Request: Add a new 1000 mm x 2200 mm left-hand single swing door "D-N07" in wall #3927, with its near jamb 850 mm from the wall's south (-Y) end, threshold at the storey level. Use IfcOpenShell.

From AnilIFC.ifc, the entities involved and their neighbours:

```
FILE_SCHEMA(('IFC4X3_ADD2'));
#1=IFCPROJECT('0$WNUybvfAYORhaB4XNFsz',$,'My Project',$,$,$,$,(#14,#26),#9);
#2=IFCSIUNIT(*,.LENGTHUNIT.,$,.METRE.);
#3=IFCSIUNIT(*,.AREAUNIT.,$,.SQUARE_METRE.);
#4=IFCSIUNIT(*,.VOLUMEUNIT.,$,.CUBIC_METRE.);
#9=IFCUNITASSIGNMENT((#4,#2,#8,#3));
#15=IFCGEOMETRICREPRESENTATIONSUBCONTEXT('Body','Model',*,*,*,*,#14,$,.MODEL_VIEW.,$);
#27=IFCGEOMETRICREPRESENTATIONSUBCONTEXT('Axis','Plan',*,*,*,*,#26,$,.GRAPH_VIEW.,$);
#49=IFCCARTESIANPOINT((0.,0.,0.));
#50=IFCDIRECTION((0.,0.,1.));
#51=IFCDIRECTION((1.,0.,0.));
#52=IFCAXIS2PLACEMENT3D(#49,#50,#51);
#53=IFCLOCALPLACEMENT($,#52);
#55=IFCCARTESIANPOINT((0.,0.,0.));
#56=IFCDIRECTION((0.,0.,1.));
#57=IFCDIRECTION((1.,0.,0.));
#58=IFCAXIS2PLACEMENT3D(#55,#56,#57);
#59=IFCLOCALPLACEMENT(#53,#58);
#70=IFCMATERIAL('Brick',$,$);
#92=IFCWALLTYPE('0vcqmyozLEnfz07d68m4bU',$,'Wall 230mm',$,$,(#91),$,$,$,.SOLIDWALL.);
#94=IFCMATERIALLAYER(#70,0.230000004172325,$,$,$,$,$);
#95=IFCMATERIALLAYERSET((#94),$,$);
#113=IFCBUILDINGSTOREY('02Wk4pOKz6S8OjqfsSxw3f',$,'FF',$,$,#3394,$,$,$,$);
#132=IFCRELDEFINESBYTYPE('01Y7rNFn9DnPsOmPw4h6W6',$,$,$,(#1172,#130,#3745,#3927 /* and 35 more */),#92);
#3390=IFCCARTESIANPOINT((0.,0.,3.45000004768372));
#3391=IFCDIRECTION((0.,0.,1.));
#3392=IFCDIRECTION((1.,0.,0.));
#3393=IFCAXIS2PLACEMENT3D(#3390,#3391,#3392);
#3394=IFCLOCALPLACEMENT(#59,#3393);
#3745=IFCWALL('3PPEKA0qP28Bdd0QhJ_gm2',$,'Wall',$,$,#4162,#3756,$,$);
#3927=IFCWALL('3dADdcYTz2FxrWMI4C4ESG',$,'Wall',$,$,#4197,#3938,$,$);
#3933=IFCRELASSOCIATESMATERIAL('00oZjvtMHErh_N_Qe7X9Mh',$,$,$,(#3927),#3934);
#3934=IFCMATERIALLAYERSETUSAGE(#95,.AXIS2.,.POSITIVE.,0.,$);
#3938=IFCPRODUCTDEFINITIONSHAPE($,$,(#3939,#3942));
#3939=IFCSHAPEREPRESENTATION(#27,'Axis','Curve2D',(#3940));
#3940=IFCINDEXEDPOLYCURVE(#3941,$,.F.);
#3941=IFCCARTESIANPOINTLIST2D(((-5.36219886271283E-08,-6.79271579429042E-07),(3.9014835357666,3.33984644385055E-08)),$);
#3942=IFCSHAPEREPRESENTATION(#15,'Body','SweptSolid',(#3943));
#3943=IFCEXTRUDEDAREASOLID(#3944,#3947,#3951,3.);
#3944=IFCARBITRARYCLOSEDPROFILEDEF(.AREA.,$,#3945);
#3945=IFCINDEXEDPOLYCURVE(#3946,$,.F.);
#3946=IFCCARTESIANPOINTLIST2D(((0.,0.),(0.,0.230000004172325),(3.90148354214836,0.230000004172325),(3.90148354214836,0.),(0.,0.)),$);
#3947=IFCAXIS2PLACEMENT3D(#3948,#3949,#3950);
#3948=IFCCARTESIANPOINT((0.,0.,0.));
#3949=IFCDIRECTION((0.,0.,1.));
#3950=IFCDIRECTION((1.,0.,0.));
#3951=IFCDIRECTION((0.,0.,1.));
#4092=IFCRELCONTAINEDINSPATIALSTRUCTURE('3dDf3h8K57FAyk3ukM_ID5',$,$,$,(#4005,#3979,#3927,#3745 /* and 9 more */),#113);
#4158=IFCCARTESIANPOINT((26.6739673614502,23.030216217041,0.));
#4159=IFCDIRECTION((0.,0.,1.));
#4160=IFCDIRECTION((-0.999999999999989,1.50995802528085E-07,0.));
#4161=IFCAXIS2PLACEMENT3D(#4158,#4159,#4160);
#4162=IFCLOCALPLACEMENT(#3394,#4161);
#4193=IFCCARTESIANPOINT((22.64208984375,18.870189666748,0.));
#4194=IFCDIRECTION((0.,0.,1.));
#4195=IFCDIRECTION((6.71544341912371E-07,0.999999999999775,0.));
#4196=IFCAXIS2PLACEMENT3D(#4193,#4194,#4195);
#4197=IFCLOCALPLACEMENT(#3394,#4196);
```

```python
import numpy as np
import ifcopenshell
import ifcopenshell.api.feature
import ifcopenshell.api.geometry
import ifcopenshell.api.root
import ifcopenshell.api.spatial
import ifcopenshell.geom
import ifcopenshell.util.element
import ifcopenshell.util.placement
import ifcopenshell.util.representation
import ifcopenshell.util.shape
import ifcopenshell.util.unit

model = ifcopenshell.open("AnilIFC.ifc")
unit_scale = ifcopenshell.util.unit.calculate_unit_scale(model)
settings = ifcopenshell.geom.settings()


def volume(element):
    """Net volume in cubic metres, openings subtracted."""
    shape = ifcopenshell.geom.create_shape(settings, element)
    return ifcopenshell.util.shape.get_volume(shape.geometry)


wall = model.by_id(3927)
storey = ifcopenshell.util.element.get_container(wall, ifc_class="IfcBuildingStorey")
context = ifcopenshell.util.representation.get_context(model, "Model", "Body", "MODEL_VIEW")
before = volume(wall)

width, height, from_end, sill = 1, 2.2, 0.85, 0.0  # metres

# The wall runs along its own X axis, and the end named is its -X end.
wall_shape = ifcopenshell.geom.create_shape(settings, wall)
x, y, z = ifcopenshell.util.shape.get_vertices(wall_shape.geometry).T
start = x.min() + from_end
face, thickness = float(y.min()), float(y.max() - y.min())
wall_matrix = ifcopenshell.util.placement.get_local_placement(wall.ObjectPlacement)
level = ifcopenshell.util.placement.get_local_placement(storey.ObjectPlacement)[2, 3]


def in_wall(x, y):
    """Placement at x, y metres in the wall's axes, at sill height."""
    matrix = wall_matrix.copy()
    matrix[:, 3] = wall_matrix @ np.array([x / unit_scale, y / unit_scale, 0.0, 1.0])
    matrix[2, 3] = level + sill / unit_scale
    return matrix


# Opening: a box that overshoots both wall faces by 50 mm.
opening = ifcopenshell.api.root.create_entity(model, ifc_class="IfcOpeningElement", predefined_type="OPENING")
box = ifcopenshell.api.geometry.add_wall_representation(
    model, context=context, length=width, height=height, thickness=thickness + 0.1
)
ifcopenshell.api.geometry.assign_representation(model, product=opening, representation=box)
ifcopenshell.api.geometry.edit_object_placement(model, product=opening, matrix=in_wall(start, face - 0.05), is_si=False)
ifcopenshell.api.feature.add_feature(model, feature=opening, element=wall)

door = ifcopenshell.api.root.create_entity(model, ifc_class="IfcDoor", name="D-N07", predefined_type="DOOR")
door.OverallWidth, door.OverallHeight = width / unit_scale, height / unit_scale
door.OperationType = "SINGLE_SWING_LEFT"
body = ifcopenshell.api.geometry.add_door_representation(
    model,
    context=context,
    overall_width=door.OverallWidth,
    overall_height=door.OverallHeight,
    operation_type="SINGLE_SWING_LEFT",
    lining_properties={"LiningDepth": thickness / unit_scale, "ThresholdDepth": thickness / unit_scale},
)
ifcopenshell.api.geometry.assign_representation(model, product=door, representation=body)
ifcopenshell.api.spatial.assign_container(model, products=[door], relating_structure=storey)
ifcopenshell.api.feature.add_filling(model, opening=opening, element=door)

# The lining spans the wall, so the door starts at the wall face.
ifcopenshell.api.geometry.edit_object_placement(model, product=door, matrix=in_wall(start, face), is_si=False)

after = volume(wall)

print(f"wall volume {before:.3f} -> {after:.3f} m3")

model.write("AnilIFC_v2.ifc")
```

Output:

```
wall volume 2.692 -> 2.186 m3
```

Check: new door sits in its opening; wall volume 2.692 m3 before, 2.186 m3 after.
